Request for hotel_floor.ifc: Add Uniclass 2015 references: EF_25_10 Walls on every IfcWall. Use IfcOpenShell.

First a look at what the model holds.

```python
import ifcopenshell

model = ifcopenshell.open("hotel_floor.ifc")
print(model.schema)
print("classifications:", [c.Name for c in model.by_type("IfcClassification")])
for ifc_class in ("IfcDoor", "IfcRoof", "IfcStair", "IfcWall", "IfcWindow"):
    print(ifc_class, len(model.by_type(ifc_class)))
```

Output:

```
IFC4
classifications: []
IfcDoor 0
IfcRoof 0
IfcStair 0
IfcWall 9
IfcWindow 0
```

```python
import ifcopenshell
import ifcopenshell.api.classification

model = ifcopenshell.open("hotel_floor.ifc")

system = ifcopenshell.api.classification.add_classification(model, classification="Uniclass 2015")

codes = {
    "IfcWall": ("EF_25_10", "Walls"),
}
for ifc_class, (code, name) in codes.items():
    products = model.by_type(ifc_class)
    ifcopenshell.api.classification.add_reference(
        model, products=products, classification=system, identification=code, name=name
    )
    print(code, len(products))

model.write("hotel_floor_v2.ifc")
```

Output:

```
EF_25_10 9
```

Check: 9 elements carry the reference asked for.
